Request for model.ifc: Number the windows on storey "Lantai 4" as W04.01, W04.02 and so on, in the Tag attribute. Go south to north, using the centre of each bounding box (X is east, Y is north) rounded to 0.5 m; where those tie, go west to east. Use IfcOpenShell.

First a look at what the model holds.

```python
import ifcopenshell
import ifcopenshell.util.element
import ifcopenshell.util.placement

model = ifcopenshell.open("model.ifc")
print(model.schema)
storey = next(s for s in model.by_type("IfcBuildingStorey") if s.Name == "Lantai 4")
windows = [e for e in ifcopenshell.util.element.get_decomposition(storey) if e.is_a("IfcWindow")]
for e in sorted(windows, key=lambda e: e.id()):
    origin = ifcopenshell.util.placement.get_local_placement(e.ObjectPlacement)[:3, 3]
    print(e.id(), e.Tag, e.Name, origin.round(2) + 0.0, sep=" | ")
```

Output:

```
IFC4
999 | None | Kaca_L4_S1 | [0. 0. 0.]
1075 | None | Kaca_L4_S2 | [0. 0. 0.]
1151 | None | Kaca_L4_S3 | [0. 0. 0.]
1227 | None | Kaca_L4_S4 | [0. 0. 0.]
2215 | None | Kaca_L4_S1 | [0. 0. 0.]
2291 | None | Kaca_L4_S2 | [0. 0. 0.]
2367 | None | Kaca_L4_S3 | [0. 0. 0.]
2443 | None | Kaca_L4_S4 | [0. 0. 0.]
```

```python
import ifcopenshell
import ifcopenshell.geom
import ifcopenshell.util.element
import ifcopenshell.util.shape

model = ifcopenshell.open("model.ifc")
settings = ifcopenshell.geom.settings()
settings.set("use-world-coords", True)


def centre(element):
    shape = ifcopenshell.geom.create_shape(settings, element)
    return ifcopenshell.util.shape.get_bbox_centroid(shape.geometry)


storey = next(s for s in model.by_type("IfcBuildingStorey") if s.Name == "Lantai 4")
windows = [e for e in ifcopenshell.util.element.get_decomposition(storey) if e.is_a("IfcWindow")]

# Insertion points can sit at a corner or the storey origin, so sort by the geometry (in metres).
centres = {e: centre(e) for e in windows}
windows.sort(key=lambda e: (round(centres[e][1] / 0.5), centres[e][0]))

for i, e in enumerate(windows, start=1):
    number = f"W04.{i:02d}"
    e.Tag = number
    print(e.id(), number)

model.write("model_v2.ifc")
```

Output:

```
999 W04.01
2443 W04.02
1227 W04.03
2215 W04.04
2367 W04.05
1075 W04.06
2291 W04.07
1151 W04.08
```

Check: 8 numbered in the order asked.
